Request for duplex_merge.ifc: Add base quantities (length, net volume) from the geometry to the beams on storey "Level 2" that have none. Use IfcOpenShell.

First a look at what the model holds.

```python
import ifcopenshell
import ifcopenshell.util.element
import ifcopenshell.util.unit

model = ifcopenshell.open("duplex_merge.ifc")
print(model.schema)
for unit_type in ("LENGTHUNIT", "AREAUNIT", "VOLUMEUNIT"):
    print(unit_type, ifcopenshell.util.unit.calculate_unit_scale(model, unit_type))
storey = next(s for s in model.by_type("IfcBuildingStorey") if s.Name == "Level 2")
beams = [e for e in ifcopenshell.util.element.get_decomposition(storey) if e.is_a("IfcBeam")]
for e in sorted(beams, key=lambda e: e.id()):
    print(e.id(), e.is_a(), e.Name, list(ifcopenshell.util.element.get_psets(e, qtos_only=True)), sep=" | ")
```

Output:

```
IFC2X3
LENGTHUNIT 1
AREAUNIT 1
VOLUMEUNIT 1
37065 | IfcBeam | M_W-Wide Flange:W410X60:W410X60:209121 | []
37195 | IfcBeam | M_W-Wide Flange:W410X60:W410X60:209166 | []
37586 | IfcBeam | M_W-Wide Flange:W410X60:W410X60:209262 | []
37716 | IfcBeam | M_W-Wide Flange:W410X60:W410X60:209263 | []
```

```python
import ifcopenshell
import ifcopenshell.api.pset
import ifcopenshell.geom
import ifcopenshell.util.element
import ifcopenshell.util.shape
import ifcopenshell.util.unit

model = ifcopenshell.open("duplex_merge.ifc")
unit_scale = ifcopenshell.util.unit.calculate_unit_scale(model)
volume_scale = ifcopenshell.util.unit.calculate_unit_scale(model, "VOLUMEUNIT")
settings = ifcopenshell.geom.settings()

storey = next(s for s in model.by_type("IfcBuildingStorey") if s.Name == "Level 2")
beams = [e for e in ifcopenshell.util.element.get_decomposition(storey) if e.is_a("IfcBeam")]

for e in sorted(beams, key=lambda e: e.id()):
    if ifcopenshell.util.element.get_psets(e, qtos_only=True, should_inherit=False):
        continue
    # Geometry comes back in metres, in the element's own axes.
    shape = ifcopenshell.geom.create_shape(settings, e)
    values = {
        "Length": ifcopenshell.util.shape.get_max_xyz(shape.geometry) / unit_scale,
        "NetVolume": ifcopenshell.util.shape.get_volume(shape.geometry) / volume_scale,
    }
    qto = ifcopenshell.api.pset.add_qto(model, product=e, name="BaseQuantities")
    ifcopenshell.api.pset.edit_qto(model, qto=qto, properties=values)
    print(e.id(), {k: round(v, 3) for k, v in values.items()})

model.write("duplex_merge_rev.ifc")
```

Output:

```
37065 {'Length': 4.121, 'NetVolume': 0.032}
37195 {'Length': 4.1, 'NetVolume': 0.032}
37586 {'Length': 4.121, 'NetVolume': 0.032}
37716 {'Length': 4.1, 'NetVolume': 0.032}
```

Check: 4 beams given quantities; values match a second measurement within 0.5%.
